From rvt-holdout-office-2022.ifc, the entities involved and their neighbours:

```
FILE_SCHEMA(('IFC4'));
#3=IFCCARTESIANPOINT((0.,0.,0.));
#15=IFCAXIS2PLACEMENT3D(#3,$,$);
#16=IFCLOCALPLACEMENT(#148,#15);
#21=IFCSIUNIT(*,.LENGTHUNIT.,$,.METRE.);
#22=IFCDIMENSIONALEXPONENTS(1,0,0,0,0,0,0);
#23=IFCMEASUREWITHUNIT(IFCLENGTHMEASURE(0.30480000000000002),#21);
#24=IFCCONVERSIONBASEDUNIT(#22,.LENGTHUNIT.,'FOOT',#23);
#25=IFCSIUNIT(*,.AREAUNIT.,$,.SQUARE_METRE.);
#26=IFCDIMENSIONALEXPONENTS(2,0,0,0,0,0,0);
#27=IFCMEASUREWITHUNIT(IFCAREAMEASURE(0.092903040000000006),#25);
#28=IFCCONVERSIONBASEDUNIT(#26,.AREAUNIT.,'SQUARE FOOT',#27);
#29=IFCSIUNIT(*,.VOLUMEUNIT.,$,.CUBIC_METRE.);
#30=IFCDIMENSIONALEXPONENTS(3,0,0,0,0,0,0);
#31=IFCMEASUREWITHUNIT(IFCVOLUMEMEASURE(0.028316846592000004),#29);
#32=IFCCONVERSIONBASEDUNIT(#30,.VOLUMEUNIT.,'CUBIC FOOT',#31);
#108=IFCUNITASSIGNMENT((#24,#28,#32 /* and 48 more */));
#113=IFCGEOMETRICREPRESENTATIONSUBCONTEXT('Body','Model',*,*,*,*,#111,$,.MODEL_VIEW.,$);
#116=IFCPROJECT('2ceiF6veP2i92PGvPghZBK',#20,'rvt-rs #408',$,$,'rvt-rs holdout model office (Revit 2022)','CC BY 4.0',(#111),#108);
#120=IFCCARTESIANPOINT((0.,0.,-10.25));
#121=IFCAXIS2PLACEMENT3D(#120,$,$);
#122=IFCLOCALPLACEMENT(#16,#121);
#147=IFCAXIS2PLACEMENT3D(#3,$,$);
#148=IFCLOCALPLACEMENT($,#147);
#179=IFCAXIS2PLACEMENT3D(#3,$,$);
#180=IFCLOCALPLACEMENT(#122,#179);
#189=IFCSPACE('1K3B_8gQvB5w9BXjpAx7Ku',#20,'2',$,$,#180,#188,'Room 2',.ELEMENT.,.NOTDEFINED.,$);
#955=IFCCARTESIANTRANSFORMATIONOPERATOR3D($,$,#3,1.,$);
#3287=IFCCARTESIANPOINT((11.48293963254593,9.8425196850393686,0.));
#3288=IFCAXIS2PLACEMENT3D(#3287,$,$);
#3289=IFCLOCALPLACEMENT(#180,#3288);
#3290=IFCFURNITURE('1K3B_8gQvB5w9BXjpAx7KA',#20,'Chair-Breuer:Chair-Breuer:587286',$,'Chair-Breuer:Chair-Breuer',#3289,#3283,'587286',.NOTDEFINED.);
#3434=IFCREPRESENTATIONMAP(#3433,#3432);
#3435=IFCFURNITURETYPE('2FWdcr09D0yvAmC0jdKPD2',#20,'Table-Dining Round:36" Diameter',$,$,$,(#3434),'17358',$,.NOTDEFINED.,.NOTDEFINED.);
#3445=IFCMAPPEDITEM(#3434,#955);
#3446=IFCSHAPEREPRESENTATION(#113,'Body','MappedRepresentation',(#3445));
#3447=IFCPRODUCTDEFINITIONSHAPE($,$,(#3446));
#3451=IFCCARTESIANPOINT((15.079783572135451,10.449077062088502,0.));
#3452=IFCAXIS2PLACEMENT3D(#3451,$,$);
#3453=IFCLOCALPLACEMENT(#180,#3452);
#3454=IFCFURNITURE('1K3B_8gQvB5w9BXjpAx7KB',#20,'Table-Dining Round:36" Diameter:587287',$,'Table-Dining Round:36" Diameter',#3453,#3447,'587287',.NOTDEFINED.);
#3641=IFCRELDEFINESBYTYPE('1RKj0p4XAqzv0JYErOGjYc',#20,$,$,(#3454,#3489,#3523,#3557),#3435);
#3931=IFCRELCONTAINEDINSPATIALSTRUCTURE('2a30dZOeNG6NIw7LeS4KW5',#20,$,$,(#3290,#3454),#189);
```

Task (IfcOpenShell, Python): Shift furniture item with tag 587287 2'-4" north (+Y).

```python
import ifcopenshell
import ifcopenshell.api.geometry
import ifcopenshell.util.placement
import ifcopenshell.util.unit

model = ifcopenshell.open("rvt-holdout-office-2022.ifc")
unit_scale = ifcopenshell.util.unit.calculate_unit_scale(model)

item = model.by_guid("1K3B_8gQvB5w9BXjpAx7KB")
matrix = ifcopenshell.util.placement.get_local_placement(item.ObjectPlacement)
matrix[1, 3] += 28 * 0.0254 / unit_scale
ifcopenshell.api.geometry.edit_object_placement(model, product=item, matrix=matrix, is_si=False)

print(ifcopenshell.util.placement.get_local_placement(item.ObjectPlacement).round(3) + 0.0)

model.write("rvt-holdout-office-2022-out.ifc")
```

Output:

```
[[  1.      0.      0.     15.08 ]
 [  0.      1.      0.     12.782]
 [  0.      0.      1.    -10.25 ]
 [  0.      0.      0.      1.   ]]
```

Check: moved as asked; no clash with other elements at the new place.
